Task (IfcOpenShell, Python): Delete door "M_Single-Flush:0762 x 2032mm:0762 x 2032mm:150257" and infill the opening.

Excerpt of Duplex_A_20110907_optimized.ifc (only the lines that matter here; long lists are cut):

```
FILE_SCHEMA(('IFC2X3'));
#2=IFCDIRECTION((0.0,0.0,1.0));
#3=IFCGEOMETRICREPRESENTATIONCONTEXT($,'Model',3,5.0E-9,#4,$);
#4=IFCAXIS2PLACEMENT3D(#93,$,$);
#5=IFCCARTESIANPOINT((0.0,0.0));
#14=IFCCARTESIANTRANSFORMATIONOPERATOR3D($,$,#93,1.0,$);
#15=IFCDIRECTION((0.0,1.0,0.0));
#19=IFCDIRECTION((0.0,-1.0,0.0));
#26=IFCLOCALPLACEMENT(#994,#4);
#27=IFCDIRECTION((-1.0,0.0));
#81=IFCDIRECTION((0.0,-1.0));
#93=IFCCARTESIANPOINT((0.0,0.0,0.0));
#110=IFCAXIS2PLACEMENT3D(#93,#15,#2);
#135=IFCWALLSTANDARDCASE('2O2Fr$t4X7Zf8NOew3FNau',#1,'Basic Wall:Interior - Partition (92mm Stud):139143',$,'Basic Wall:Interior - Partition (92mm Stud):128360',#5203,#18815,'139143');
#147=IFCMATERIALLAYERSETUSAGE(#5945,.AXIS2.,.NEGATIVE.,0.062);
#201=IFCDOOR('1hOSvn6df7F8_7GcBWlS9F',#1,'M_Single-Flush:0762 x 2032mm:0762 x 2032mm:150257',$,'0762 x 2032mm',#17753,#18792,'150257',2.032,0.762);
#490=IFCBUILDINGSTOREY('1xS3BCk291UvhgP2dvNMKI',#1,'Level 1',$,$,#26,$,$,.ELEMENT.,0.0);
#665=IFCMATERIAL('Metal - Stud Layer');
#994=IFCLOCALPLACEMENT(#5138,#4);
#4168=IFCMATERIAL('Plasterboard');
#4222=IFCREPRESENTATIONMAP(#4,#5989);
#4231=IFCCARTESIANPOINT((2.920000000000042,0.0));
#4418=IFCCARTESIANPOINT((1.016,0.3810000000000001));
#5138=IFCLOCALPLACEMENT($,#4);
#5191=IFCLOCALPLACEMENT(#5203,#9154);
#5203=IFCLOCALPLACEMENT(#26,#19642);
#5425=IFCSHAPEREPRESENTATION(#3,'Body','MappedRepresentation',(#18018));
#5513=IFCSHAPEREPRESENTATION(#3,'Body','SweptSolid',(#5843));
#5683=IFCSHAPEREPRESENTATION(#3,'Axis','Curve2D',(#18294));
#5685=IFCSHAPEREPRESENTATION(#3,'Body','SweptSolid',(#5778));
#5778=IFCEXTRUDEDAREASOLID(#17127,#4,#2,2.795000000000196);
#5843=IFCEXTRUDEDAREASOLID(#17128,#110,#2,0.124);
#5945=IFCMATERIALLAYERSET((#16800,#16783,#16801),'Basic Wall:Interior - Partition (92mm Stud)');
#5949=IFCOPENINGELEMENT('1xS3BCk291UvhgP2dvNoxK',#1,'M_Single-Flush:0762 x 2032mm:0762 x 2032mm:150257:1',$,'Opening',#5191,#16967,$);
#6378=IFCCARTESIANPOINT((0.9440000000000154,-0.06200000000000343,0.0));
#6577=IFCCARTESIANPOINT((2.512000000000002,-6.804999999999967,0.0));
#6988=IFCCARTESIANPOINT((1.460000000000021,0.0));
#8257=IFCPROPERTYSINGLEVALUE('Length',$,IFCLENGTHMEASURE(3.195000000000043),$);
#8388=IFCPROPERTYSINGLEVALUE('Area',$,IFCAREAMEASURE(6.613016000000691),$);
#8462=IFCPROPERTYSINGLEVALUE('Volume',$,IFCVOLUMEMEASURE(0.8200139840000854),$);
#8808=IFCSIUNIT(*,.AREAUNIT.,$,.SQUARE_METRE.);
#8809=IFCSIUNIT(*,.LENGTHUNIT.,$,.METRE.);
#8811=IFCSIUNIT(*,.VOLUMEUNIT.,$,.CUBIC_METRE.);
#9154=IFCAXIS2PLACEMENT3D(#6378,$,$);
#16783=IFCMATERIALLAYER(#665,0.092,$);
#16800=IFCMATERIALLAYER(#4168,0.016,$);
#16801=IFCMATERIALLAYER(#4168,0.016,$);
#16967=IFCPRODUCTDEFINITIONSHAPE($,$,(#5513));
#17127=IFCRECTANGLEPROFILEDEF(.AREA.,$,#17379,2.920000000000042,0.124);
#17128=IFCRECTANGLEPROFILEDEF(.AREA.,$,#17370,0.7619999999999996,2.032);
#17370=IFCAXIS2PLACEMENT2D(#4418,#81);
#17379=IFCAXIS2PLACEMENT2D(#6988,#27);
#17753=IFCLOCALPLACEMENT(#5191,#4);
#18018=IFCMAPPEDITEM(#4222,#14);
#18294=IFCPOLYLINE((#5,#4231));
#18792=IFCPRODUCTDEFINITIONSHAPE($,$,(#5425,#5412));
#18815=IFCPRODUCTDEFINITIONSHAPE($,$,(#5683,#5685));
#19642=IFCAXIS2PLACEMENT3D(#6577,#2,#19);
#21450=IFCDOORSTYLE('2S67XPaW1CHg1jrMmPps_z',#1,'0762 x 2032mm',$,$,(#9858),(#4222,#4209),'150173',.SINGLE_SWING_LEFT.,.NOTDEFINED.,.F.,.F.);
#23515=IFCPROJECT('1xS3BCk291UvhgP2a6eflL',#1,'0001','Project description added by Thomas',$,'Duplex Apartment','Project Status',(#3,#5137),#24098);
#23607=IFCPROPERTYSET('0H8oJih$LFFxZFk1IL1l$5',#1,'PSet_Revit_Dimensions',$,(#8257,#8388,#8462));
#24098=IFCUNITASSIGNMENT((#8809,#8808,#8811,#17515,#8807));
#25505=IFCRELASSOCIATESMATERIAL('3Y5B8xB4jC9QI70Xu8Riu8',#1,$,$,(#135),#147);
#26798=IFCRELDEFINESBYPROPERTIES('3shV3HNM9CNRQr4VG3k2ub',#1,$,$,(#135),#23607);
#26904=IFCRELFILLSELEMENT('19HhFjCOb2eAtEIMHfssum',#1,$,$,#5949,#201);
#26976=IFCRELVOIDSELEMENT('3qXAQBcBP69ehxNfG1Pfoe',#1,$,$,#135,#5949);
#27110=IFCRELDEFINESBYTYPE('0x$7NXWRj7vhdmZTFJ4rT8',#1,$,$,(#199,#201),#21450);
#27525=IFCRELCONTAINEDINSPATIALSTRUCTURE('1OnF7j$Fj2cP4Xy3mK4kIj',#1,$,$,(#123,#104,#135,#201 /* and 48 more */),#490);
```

```python
import ifcopenshell
import ifcopenshell.api.feature
import ifcopenshell.api.pset
import ifcopenshell.api.root
import ifcopenshell.geom
import ifcopenshell.util.element
import ifcopenshell.util.shape
import ifcopenshell.util.unit

model = ifcopenshell.open("Duplex_A_20110907_optimized.ifc")
area_scale = ifcopenshell.util.unit.calculate_unit_scale(model, "AREAUNIT")
volume_scale = ifcopenshell.util.unit.calculate_unit_scale(model, "VOLUMEUNIT")
settings = ifcopenshell.geom.settings()


def volume(element):
    """Net volume in cubic metres, openings subtracted."""
    shape = ifcopenshell.geom.create_shape(settings, element)
    return ifcopenshell.util.shape.get_volume(shape.geometry)


door = model.by_guid("1hOSvn6df7F8_7GcBWlS9F")
opening = door.FillsVoids[0].RelatingOpeningElement
wall = opening.VoidsElements[0].RelatingBuildingElement
before = volume(wall)

ifcopenshell.api.root.remove_product(model, product=door)
ifcopenshell.api.feature.remove_feature(model, feature=opening)

after = volume(wall)
thickness = 0.124  # wall thickness in metres

# Update the wall's stored quantities.
pset = model.by_id(ifcopenshell.util.element.get_pset(wall, "PSet_Revit_Dimensions", should_inherit=False)["id"])
ifcopenshell.api.pset.edit_pset(model, pset=pset, properties={
    "Area": model.create_entity("IfcAreaMeasure", after / thickness / area_scale),
    "Volume": model.create_entity("IfcVolumeMeasure", after / volume_scale),
})

print(f"wall volume {before:.3f} -> {after:.3f} m3")

model.write("Duplex_A_20110907_optimized_updated.ifc")
```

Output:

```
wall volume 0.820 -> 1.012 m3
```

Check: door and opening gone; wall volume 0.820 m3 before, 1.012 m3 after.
